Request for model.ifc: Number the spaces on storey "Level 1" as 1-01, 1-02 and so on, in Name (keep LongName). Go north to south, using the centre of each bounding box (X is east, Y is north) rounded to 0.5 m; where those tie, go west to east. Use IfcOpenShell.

First a look at what the model holds.

```python
import ifcopenshell
import ifcopenshell.util.element
import ifcopenshell.util.placement

model = ifcopenshell.open("model.ifc")
print(model.schema)
storey = next(s for s in model.by_type("IfcBuildingStorey") if s.Name == "Level 1")
spaces = [e for e in ifcopenshell.util.element.get_decomposition(storey) if e.is_a("IfcSpace")]
for e in sorted(spaces, key=lambda e: e.id()):
    origin = ifcopenshell.util.placement.get_local_placement(e.ObjectPlacement)[:3, 3]
    print(e.id(), e.Name, e.LongName, origin.round(2) + 0.0, sep=" | ")
```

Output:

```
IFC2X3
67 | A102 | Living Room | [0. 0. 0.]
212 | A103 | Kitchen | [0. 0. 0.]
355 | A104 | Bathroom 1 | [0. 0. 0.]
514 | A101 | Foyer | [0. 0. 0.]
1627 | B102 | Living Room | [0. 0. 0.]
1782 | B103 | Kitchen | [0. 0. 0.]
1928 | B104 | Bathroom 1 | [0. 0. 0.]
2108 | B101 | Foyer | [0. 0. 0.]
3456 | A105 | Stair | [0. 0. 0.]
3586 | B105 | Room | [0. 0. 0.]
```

```python
import ifcopenshell
import ifcopenshell.geom
import ifcopenshell.util.element
import ifcopenshell.util.shape

model = ifcopenshell.open("model.ifc")
settings = ifcopenshell.geom.settings()
settings.set("use-world-coords", True)


def centre(element):
    shape = ifcopenshell.geom.create_shape(settings, element)
    return ifcopenshell.util.shape.get_bbox_centroid(shape.geometry)


storey = next(s for s in model.by_type("IfcBuildingStorey") if s.Name == "Level 1")
spaces = [e for e in ifcopenshell.util.element.get_decomposition(storey) if e.is_a("IfcSpace")]

# Insertion points can sit at a corner or the storey origin, so sort by the geometry (in metres).
centres = {e: centre(e) for e in spaces}
spaces.sort(key=lambda e: (-round(centres[e][1] / 0.5), centres[e][0]))

for i, e in enumerate(spaces, start=1):
    number = f"1-{i:02d}"
    e.Name = number
    print(e.id(), number)

model.write("model-out.ifc")
```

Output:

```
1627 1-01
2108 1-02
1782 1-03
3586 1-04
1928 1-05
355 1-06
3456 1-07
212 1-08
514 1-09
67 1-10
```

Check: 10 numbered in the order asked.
